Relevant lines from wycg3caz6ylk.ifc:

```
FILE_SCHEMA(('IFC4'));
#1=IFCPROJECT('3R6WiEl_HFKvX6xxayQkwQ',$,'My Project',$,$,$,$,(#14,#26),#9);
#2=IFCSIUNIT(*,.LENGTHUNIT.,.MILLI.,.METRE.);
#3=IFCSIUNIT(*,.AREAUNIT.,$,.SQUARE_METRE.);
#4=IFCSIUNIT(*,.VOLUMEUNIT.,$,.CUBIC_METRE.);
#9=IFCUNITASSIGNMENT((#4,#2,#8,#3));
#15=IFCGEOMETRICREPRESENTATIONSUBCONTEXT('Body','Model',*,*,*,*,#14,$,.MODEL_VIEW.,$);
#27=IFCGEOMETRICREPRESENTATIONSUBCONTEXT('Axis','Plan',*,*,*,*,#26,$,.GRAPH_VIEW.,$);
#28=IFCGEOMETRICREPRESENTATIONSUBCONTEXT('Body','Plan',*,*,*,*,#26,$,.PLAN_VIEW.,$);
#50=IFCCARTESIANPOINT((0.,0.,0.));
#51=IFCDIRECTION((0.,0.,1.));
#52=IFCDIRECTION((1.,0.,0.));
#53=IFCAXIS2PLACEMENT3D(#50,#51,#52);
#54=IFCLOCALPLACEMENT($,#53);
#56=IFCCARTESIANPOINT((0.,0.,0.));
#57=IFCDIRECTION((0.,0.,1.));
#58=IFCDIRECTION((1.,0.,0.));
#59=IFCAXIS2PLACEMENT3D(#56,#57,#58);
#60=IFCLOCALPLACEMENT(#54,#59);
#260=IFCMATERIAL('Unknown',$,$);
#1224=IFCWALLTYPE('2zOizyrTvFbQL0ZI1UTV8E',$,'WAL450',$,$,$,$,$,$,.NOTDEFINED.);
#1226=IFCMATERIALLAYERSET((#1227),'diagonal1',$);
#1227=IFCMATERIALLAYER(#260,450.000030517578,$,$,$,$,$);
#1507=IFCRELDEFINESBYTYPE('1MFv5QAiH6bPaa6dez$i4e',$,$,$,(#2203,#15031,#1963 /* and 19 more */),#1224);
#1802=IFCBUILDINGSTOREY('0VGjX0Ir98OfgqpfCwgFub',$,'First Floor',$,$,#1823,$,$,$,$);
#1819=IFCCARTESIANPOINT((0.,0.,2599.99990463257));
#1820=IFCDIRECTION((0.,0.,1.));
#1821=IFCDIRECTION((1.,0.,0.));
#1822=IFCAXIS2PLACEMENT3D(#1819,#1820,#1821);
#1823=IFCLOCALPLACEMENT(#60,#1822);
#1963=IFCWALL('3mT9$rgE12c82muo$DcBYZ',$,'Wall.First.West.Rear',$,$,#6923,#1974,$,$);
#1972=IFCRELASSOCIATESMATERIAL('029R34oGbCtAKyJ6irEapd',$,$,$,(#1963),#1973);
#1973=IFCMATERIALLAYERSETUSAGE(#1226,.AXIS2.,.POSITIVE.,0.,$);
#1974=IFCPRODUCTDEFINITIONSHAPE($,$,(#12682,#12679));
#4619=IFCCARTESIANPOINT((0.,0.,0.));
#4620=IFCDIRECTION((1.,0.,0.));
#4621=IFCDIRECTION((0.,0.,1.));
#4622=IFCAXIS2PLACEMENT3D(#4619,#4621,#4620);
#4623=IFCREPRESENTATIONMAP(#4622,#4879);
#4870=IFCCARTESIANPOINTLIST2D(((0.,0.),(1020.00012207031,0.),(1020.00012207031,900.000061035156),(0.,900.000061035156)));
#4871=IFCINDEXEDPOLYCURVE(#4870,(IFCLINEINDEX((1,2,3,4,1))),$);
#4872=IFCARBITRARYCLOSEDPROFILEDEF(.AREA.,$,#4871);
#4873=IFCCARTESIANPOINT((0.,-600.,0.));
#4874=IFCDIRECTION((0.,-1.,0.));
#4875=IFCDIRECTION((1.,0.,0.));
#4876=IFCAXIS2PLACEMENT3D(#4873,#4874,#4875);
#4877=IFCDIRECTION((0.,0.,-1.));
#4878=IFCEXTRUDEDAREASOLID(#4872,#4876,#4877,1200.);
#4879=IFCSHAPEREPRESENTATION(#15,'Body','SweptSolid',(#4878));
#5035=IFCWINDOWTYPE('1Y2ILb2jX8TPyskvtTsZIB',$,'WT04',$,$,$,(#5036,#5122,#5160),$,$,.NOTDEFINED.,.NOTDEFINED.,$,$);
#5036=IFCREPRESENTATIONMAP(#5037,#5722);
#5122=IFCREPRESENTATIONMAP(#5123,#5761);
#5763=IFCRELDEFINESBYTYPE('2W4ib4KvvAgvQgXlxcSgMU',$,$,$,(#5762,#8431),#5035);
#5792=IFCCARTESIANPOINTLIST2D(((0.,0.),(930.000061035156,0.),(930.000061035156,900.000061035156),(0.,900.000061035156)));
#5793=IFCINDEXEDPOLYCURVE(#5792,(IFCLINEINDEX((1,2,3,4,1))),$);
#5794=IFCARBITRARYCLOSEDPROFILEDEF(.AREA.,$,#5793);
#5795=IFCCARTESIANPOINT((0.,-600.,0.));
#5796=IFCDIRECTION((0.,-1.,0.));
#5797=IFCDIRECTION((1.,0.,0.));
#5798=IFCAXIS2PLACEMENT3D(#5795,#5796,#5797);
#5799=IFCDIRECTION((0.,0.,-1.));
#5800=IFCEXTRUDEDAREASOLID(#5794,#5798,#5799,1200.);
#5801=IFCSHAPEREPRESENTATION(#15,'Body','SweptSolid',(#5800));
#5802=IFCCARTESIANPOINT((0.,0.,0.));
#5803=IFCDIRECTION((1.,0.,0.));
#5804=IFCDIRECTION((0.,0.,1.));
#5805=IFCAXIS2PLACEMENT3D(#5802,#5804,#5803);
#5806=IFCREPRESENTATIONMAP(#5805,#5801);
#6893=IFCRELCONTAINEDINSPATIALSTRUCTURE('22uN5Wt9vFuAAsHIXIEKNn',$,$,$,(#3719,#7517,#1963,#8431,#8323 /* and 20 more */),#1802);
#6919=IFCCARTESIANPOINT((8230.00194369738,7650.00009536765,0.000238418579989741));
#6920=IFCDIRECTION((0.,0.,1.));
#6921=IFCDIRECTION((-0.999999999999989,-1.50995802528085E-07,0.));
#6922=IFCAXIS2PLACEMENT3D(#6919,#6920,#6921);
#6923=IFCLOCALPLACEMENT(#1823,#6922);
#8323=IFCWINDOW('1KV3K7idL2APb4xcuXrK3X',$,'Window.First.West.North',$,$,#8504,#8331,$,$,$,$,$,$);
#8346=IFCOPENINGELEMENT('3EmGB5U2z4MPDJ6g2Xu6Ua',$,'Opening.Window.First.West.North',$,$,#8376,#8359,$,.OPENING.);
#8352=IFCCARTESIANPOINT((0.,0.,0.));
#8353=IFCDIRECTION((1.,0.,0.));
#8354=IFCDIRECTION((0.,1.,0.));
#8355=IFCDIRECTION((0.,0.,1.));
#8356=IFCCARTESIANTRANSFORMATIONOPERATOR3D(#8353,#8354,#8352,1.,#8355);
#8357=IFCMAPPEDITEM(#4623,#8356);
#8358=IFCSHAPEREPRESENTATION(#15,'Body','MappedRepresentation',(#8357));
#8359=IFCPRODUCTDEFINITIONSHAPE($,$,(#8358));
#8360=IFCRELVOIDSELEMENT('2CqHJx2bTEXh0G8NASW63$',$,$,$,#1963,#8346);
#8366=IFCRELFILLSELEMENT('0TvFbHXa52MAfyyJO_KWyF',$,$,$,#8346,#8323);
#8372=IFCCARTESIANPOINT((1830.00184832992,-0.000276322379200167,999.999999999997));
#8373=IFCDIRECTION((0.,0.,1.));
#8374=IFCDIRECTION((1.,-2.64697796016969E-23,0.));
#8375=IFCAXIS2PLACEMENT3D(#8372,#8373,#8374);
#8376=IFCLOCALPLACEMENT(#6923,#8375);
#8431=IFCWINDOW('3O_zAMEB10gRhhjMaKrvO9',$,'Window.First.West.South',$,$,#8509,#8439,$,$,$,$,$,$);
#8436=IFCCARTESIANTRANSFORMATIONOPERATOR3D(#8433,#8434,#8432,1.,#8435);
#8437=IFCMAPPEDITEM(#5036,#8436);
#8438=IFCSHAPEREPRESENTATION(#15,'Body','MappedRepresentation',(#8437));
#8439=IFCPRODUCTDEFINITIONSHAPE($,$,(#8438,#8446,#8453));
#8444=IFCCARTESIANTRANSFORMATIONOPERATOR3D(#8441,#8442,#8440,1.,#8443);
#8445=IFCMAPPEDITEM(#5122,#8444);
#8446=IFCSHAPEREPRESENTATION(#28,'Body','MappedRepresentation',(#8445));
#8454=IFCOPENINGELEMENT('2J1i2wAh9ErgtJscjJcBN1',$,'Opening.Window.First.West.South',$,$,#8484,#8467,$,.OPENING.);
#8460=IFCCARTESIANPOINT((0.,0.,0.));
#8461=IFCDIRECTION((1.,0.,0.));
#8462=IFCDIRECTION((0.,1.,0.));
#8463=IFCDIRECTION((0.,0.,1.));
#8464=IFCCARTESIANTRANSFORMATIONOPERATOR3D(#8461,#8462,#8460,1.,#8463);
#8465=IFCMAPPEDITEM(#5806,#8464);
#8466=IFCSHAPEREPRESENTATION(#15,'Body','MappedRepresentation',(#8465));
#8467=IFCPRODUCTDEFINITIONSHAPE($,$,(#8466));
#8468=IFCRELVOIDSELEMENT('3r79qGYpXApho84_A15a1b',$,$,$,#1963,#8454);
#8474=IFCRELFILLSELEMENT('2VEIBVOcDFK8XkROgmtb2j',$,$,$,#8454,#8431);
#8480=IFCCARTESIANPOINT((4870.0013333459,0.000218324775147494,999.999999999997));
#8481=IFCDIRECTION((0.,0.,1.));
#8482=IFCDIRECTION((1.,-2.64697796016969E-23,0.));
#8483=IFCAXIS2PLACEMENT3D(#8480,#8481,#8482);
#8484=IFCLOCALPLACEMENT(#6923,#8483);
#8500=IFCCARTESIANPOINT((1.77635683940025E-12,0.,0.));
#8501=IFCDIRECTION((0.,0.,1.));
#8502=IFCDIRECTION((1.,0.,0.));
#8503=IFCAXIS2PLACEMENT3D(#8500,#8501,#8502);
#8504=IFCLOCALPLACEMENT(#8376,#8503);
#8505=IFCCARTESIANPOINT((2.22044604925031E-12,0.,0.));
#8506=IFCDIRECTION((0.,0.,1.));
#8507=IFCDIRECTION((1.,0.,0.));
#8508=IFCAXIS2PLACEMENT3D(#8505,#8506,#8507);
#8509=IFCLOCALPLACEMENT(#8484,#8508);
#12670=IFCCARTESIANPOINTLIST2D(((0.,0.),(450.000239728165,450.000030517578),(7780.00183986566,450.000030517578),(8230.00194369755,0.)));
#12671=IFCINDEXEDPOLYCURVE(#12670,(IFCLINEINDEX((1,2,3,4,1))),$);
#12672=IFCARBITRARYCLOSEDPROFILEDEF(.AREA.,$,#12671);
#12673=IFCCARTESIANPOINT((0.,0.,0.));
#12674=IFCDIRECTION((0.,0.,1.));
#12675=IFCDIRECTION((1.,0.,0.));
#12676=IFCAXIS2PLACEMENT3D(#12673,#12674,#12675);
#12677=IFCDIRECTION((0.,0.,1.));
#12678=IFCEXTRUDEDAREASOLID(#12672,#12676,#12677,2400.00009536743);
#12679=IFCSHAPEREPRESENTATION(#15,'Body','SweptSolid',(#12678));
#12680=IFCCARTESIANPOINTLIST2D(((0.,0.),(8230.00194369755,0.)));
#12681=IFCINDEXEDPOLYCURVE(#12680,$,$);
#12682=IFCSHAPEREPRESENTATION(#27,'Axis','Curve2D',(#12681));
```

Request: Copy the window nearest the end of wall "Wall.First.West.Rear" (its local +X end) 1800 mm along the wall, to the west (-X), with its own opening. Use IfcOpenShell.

```python
import ifcopenshell
import ifcopenshell.api.feature
import ifcopenshell.api.geometry
import ifcopenshell.api.root
import ifcopenshell.geom
import ifcopenshell.util.element
import ifcopenshell.util.placement
import ifcopenshell.util.shape
import ifcopenshell.util.unit

model = ifcopenshell.open("wycg3caz6ylk.ifc")
unit_scale = ifcopenshell.util.unit.calculate_unit_scale(model)
settings = ifcopenshell.geom.settings()


def volume(element):
    """Net volume in cubic metres, openings subtracted."""
    shape = ifcopenshell.geom.create_shape(settings, element)
    return ifcopenshell.util.shape.get_volume(shape.geometry)


window = model.by_guid("3O_zAMEB10gRhhjMaKrvO9")
opening = window.FillsVoids[0].RelatingOpeningElement
wall = opening.VoidsElements[0].RelatingBuildingElement
before = volume(wall)
shift = ifcopenshell.util.placement.get_local_placement(wall.ObjectPlacement)[:3, 0] * 1.8 / unit_scale

# copy_class copies the void relationship, type, container and properties, but no geometry.
new_opening = ifcopenshell.api.root.copy_class(model, product=opening)
new_opening.Representation = ifcopenshell.util.element.copy_deep(
    model, opening.Representation, exclude=["IfcGeometricRepresentationContext", "IfcRepresentationMap"]
)
new_window = ifcopenshell.api.root.copy_class(model, product=window)
new_window.Representation = ifcopenshell.util.element.copy_deep(
    model, window.Representation, exclude=["IfcGeometricRepresentationContext", "IfcRepresentationMap"]
)
ifcopenshell.api.feature.add_filling(model, opening=new_opening, element=new_window)

for old, new in ((opening, new_opening), (window, new_window)):
    matrix = ifcopenshell.util.placement.get_local_placement(old.ObjectPlacement)
    matrix[:3, 3] += shift
    ifcopenshell.api.geometry.edit_object_placement(model, product=new, matrix=matrix, is_si=False)

after = volume(wall)

print(f"wall volume {before:.3f} -> {after:.3f} m3")

model.write("wycg3caz6ylk_rev.ifc")
```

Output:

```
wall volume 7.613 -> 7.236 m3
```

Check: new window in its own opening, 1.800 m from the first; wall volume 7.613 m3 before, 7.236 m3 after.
